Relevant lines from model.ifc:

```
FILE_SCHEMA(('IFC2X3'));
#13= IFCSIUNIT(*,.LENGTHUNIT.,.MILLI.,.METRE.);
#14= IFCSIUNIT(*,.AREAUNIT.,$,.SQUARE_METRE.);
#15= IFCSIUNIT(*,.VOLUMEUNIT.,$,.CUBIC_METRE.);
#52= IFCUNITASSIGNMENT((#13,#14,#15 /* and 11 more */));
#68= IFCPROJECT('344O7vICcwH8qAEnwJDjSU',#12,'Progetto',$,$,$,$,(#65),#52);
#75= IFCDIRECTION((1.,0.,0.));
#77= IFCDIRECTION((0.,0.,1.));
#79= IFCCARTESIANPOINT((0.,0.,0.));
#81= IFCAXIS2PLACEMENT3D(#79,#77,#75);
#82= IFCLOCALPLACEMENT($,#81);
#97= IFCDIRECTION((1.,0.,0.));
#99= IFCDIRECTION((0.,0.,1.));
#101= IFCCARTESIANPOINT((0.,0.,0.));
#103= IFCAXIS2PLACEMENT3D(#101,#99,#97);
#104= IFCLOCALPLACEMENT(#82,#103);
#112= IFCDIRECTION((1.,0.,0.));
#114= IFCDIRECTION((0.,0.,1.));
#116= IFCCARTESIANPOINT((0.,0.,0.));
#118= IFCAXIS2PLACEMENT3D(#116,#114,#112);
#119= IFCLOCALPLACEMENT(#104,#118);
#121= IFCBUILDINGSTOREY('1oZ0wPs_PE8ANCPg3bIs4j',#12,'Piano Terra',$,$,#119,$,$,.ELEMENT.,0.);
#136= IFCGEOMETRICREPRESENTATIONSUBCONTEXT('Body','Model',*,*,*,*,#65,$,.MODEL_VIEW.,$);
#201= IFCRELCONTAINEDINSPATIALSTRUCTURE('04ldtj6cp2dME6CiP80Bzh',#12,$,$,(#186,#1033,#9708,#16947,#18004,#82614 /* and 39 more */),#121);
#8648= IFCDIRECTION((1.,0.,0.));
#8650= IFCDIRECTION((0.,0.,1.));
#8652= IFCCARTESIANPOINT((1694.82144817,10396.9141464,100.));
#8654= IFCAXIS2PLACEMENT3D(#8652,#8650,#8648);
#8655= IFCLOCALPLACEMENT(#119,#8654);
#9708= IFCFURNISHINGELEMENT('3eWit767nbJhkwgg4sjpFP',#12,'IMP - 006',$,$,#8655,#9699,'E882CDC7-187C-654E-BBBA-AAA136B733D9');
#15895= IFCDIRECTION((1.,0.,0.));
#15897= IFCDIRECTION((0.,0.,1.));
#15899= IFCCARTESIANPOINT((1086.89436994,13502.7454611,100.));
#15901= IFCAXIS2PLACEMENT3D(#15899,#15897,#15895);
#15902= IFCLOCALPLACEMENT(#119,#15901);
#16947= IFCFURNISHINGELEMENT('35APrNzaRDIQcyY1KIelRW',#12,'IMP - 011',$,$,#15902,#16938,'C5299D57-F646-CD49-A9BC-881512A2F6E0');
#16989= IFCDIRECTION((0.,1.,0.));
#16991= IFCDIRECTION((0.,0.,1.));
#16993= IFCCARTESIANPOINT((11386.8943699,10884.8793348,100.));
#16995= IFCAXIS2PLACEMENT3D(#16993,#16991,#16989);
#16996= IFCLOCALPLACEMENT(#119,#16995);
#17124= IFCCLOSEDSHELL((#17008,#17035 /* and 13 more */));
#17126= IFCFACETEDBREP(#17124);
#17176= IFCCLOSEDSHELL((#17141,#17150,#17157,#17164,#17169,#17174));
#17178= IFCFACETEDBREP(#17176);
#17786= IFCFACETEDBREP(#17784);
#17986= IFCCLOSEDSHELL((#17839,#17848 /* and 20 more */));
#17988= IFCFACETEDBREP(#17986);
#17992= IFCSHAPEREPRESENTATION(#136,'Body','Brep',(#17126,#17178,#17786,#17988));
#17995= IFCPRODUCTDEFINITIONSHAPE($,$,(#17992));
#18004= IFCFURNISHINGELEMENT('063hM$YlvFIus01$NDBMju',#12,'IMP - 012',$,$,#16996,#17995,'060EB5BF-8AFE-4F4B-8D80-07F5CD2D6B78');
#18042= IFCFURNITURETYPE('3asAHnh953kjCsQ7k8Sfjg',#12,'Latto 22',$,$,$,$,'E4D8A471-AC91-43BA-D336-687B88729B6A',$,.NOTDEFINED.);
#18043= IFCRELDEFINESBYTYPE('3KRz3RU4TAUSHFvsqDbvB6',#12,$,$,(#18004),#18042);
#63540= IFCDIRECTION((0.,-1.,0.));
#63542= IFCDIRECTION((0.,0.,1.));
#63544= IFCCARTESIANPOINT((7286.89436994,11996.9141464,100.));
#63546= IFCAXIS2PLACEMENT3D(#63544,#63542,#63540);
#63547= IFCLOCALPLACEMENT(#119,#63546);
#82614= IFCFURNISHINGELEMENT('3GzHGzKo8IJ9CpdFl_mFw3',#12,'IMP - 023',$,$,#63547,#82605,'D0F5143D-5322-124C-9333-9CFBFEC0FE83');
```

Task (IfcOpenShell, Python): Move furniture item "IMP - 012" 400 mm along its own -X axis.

```python
import ifcopenshell
import ifcopenshell.api.geometry
import ifcopenshell.util.placement

model = ifcopenshell.open("model.ifc")

item = model.by_id(18004)
matrix = ifcopenshell.util.placement.get_local_placement(item.ObjectPlacement)
matrix[:3, 3] -= matrix[:3, 0] * 400.0
ifcopenshell.api.geometry.edit_object_placement(model, product=item, matrix=matrix, is_si=False)

print(ifcopenshell.util.placement.get_local_placement(item.ObjectPlacement).round(3) + 0.0)

model.write("model_updated.ifc")
```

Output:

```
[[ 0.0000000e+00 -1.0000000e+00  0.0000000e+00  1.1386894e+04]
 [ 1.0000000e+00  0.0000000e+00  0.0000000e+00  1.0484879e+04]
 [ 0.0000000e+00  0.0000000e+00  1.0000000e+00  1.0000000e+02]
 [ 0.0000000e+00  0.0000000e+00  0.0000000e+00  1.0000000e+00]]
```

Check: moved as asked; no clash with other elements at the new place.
